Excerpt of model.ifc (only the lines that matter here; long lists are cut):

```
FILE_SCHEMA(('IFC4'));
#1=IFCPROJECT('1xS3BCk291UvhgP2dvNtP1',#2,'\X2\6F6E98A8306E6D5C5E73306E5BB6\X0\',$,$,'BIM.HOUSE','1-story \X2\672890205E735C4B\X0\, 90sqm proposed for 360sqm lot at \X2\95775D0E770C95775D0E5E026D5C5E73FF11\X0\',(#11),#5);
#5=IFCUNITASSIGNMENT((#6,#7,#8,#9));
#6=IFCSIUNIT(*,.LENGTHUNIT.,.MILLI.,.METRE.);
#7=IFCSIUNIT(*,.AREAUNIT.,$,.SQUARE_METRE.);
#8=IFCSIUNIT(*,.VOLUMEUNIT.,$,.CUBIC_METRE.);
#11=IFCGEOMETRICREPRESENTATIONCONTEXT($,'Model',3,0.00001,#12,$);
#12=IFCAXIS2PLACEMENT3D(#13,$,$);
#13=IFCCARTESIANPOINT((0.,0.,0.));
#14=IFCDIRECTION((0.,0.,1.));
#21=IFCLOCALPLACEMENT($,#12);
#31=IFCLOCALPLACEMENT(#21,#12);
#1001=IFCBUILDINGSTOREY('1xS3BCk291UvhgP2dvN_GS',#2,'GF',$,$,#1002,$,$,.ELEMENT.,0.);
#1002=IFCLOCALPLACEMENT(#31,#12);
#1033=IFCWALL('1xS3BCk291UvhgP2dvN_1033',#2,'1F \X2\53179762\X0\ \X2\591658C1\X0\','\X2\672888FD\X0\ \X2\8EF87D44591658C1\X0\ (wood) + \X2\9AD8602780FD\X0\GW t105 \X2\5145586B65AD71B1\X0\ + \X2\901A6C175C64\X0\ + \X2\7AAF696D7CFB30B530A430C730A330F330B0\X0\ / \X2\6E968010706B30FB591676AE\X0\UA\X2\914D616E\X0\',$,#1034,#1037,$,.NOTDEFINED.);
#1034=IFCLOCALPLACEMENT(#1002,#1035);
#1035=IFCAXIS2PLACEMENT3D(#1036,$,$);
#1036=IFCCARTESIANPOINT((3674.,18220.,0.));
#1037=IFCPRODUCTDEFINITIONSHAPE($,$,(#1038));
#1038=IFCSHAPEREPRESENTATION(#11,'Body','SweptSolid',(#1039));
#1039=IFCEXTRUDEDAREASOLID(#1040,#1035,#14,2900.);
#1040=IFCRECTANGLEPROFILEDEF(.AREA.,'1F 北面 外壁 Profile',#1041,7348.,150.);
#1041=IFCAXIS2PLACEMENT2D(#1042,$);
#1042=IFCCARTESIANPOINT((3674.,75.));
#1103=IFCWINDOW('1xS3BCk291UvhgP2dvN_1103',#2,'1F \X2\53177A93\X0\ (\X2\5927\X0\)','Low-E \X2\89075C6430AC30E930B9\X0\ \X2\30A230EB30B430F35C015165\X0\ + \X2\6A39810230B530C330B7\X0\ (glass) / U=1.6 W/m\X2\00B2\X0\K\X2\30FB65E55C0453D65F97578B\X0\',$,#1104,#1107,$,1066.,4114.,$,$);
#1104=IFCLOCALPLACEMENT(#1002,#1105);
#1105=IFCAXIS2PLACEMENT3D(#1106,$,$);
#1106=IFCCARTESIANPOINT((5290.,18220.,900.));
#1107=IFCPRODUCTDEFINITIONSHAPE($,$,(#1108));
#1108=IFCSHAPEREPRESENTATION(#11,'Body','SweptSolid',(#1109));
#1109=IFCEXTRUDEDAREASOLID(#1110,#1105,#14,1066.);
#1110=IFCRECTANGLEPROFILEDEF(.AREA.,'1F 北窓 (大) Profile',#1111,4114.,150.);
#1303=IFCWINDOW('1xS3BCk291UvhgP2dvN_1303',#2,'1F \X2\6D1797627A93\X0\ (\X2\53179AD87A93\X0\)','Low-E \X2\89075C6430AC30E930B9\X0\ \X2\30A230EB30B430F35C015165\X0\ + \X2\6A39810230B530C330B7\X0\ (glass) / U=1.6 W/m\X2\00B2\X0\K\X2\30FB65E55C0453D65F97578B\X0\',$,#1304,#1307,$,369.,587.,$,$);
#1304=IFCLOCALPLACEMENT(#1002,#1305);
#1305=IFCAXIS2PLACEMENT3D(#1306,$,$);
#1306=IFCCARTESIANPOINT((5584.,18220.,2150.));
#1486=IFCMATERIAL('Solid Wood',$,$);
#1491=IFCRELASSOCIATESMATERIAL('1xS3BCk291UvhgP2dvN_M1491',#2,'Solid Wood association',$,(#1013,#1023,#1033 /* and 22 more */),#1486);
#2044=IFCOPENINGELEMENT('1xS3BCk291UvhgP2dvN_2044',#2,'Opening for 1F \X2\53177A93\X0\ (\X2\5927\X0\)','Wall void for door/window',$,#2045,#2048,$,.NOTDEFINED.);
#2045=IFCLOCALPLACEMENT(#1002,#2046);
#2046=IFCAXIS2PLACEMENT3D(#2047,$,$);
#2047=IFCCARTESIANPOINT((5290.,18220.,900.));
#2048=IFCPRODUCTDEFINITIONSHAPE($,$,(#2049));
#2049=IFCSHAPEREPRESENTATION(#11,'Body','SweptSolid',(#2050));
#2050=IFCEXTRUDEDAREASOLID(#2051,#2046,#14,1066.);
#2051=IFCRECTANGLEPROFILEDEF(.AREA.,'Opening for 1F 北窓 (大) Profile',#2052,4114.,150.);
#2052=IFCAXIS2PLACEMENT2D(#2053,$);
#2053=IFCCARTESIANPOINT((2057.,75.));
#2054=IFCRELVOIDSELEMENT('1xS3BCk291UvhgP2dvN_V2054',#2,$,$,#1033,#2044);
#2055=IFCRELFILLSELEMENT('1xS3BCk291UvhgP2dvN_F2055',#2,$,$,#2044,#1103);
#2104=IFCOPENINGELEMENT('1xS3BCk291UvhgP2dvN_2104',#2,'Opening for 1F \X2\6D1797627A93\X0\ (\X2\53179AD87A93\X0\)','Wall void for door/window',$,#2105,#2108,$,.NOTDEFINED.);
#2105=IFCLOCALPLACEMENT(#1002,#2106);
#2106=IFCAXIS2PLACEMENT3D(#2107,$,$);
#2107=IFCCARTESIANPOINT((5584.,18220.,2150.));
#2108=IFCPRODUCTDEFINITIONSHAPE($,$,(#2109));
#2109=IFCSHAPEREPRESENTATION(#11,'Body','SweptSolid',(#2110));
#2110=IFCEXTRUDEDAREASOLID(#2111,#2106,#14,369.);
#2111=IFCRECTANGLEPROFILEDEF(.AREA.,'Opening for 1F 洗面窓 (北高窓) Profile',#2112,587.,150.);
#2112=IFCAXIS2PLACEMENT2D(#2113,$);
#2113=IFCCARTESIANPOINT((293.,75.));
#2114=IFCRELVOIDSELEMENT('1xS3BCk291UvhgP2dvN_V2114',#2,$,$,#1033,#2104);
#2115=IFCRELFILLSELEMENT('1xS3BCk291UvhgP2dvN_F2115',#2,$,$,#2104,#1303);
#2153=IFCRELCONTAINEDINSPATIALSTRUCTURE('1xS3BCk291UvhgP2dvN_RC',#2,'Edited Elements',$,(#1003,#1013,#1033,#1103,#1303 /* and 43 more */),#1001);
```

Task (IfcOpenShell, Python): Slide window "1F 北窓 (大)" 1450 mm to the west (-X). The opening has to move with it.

```python
import ifcopenshell
import ifcopenshell.api.geometry
import ifcopenshell.util.placement
import ifcopenshell.util.unit

model = ifcopenshell.open("model.ifc")
unit_scale = ifcopenshell.util.unit.calculate_unit_scale(model)

window = model.by_guid("1xS3BCk291UvhgP2dvN_1103")
opening = window.FillsVoids[0].RelatingOpeningElement
wall = opening.VoidsElements[0].RelatingBuildingElement

wall_matrix = ifcopenshell.util.placement.get_local_placement(wall.ObjectPlacement)
shift = wall_matrix[:3, 0] * -1.45 / unit_scale
before = ifcopenshell.util.placement.get_local_placement(window.ObjectPlacement)[:3, 3].copy()

# The window is not placed relative to its opening, so move both.
for product in (opening, window):
    matrix = ifcopenshell.util.placement.get_local_placement(product.ObjectPlacement)
    matrix[:3, 3] += shift
    ifcopenshell.api.geometry.edit_object_placement(model, product=product, matrix=matrix, is_si=False)

after = ifcopenshell.util.placement.get_local_placement(window.ObjectPlacement)[:3, 3]
print("window moved by", (after - before).round(3) + 0.0)

model.write("model-out.ifc")
```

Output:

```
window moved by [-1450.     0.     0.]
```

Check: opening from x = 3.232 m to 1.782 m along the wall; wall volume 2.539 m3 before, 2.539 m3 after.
